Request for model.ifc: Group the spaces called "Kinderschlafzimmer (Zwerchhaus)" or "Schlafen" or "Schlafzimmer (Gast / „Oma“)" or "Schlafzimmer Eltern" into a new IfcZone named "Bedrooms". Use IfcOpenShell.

First a look at what the model holds.

```python
import ifcopenshell

model = ifcopenshell.open("model.ifc")
print(model.schema)
seen = {}
for space in model.by_type("IfcSpace"):
    seen[space.LongName] = seen.get(space.LongName, 0) + 1
for name, count in sorted(seen.items(), key=str):
    print(count, "x", name)
print("zones:", [z.Name for z in model.by_type("IfcZone")][:20])
```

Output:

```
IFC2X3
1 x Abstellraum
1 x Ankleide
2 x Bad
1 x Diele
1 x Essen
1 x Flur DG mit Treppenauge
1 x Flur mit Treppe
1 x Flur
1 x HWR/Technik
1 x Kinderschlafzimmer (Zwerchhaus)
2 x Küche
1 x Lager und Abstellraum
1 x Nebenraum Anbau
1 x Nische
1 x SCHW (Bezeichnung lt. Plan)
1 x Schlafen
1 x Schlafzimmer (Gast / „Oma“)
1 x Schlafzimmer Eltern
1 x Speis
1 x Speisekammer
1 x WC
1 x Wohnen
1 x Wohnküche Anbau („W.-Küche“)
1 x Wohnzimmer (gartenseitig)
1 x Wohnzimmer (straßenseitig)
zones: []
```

```python
import ifcopenshell
import ifcopenshell.api.group
import ifcopenshell.api.root

model = ifcopenshell.open("model.ifc")

names = {"Kinderschlafzimmer (Zwerchhaus)", "Schlafen", "Schlafzimmer (Gast / „Oma“)", "Schlafzimmer Eltern"}
spaces = [s for s in model.by_type("IfcSpace") if s.LongName in names]

zone = ifcopenshell.api.root.create_entity(model, ifc_class="IfcZone", name="Bedrooms")
ifcopenshell.api.group.assign_group(model, products=spaces, group=zone)
print(len(spaces), "spaces in", zone.Name)

model.write("model_rev.ifc")
```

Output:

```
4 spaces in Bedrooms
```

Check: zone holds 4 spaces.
